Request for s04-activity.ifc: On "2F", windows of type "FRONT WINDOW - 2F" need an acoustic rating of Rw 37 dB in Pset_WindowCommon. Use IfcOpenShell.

First a look at what the model holds.

```python
import ifcopenshell
import ifcopenshell.util.element

model = ifcopenshell.open("s04-activity.ifc")
print(model.schema)
storey = next(s for s in model.by_type("IfcBuildingStorey") if s.Name == "2F")
windows = [e for e in ifcopenshell.util.element.get_decomposition(storey) if e.is_a("IfcWindow")]
seen = {}
for e in windows:
    element_type = ifcopenshell.util.element.get_type(e)
    key = (element_type.Name if element_type != e and element_type else None, ifcopenshell.util.element.get_pset(e, "Pset_WindowCommon", "AcousticRating"))
    seen[key] = seen.get(key, 0) + 1
for (name, value), count in sorted(seen.items(), key=str):
    print(count, "x", name, "|", value)
```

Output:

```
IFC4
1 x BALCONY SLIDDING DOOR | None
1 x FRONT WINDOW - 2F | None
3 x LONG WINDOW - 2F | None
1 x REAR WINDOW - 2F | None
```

```python
import ifcopenshell
import ifcopenshell.api.pset
import ifcopenshell.util.element

model = ifcopenshell.open("s04-activity.ifc")

storey = next(s for s in model.by_type("IfcBuildingStorey") if s.Name == "2F")
windows = [e for e in ifcopenshell.util.element.get_decomposition(storey) if e.is_a("IfcWindow")]

count = 0
for e in windows:
    element_type = ifcopenshell.util.element.get_type(e)
    if element_type in (None, e) or element_type.Name != "FRONT WINDOW - 2F":
        continue
    # add_pset returns the element's existing set when there is one.
    pset = ifcopenshell.api.pset.add_pset(model, product=e, name="Pset_WindowCommon")
    ifcopenshell.api.pset.edit_pset(model, pset=pset, properties={"AcousticRating": "Rw 37 dB"})
    count += 1

print(count, "windows updated")

model.write("s04-activity_v2.ifc")
```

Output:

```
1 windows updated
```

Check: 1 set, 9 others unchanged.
